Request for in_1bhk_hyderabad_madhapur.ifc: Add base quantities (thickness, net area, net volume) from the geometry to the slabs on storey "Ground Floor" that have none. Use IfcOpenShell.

First a look at what the model holds.

```python
import ifcopenshell
import ifcopenshell.util.element
import ifcopenshell.util.unit

model = ifcopenshell.open("in_1bhk_hyderabad_madhapur.ifc")
print(model.schema)
for unit_type in ("LENGTHUNIT", "AREAUNIT", "VOLUMEUNIT"):
    print(unit_type, ifcopenshell.util.unit.calculate_unit_scale(model, unit_type))
storey = next(s for s in model.by_type("IfcBuildingStorey") if s.Name == "Ground Floor")
slabs = [e for e in ifcopenshell.util.element.get_decomposition(storey) if e.is_a("IfcSlab")]
for e in sorted(slabs, key=lambda e: e.id()):
    print(e.id(), e.is_a(), e.Name, list(ifcopenshell.util.element.get_psets(e, qtos_only=True)), sep=" | ")
```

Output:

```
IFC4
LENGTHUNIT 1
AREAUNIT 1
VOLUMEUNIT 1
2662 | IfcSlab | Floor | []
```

```python
import ifcopenshell
import ifcopenshell.api.pset
import ifcopenshell.geom
import ifcopenshell.util.element
import ifcopenshell.util.shape
import ifcopenshell.util.unit

model = ifcopenshell.open("in_1bhk_hyderabad_madhapur.ifc")
unit_scale = ifcopenshell.util.unit.calculate_unit_scale(model)
area_scale = ifcopenshell.util.unit.calculate_unit_scale(model, "AREAUNIT")
volume_scale = ifcopenshell.util.unit.calculate_unit_scale(model, "VOLUMEUNIT")
settings = ifcopenshell.geom.settings()

storey = next(s for s in model.by_type("IfcBuildingStorey") if s.Name == "Ground Floor")
slabs = [e for e in ifcopenshell.util.element.get_decomposition(storey) if e.is_a("IfcSlab")]

for e in sorted(slabs, key=lambda e: e.id()):
    if ifcopenshell.util.element.get_psets(e, qtos_only=True, should_inherit=False):
        continue
    # Geometry comes back in metres, in the element's own axes.
    shape = ifcopenshell.geom.create_shape(settings, e)
    values = {
        "Width": ifcopenshell.util.shape.get_z(shape.geometry) / unit_scale,
        "NetArea": ifcopenshell.util.shape.get_footprint_area(shape.geometry) / area_scale,
        "NetVolume": ifcopenshell.util.shape.get_volume(shape.geometry) / volume_scale,
    }
    qto = ifcopenshell.api.pset.add_qto(model, product=e, name="Qto_SlabBaseQuantities")
    ifcopenshell.api.pset.edit_qto(model, qto=qto, properties=values)
    print(e.id(), {k: round(v, 3) for k, v in values.items()})

model.write("in_1bhk_hyderabad_madhapur_edited.ifc")
```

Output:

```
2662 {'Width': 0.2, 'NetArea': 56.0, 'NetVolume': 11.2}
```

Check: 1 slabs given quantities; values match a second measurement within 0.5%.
